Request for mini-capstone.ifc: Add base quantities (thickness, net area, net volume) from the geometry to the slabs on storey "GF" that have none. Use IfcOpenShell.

First a look at what the model holds.

```python
import ifcopenshell
import ifcopenshell.util.element
import ifcopenshell.util.unit

model = ifcopenshell.open("mini-capstone.ifc")
print(model.schema)
for unit_type in ("LENGTHUNIT", "AREAUNIT", "VOLUMEUNIT"):
    print(unit_type, ifcopenshell.util.unit.calculate_unit_scale(model, unit_type))
storey = next(s for s in model.by_type("IfcBuildingStorey") if s.Name == "GF")
slabs = [e for e in ifcopenshell.util.element.get_decomposition(storey) if e.is_a("IfcSlab")]
for e in sorted(slabs, key=lambda e: e.id()):
    print(e.id(), e.is_a(), e.Name, list(ifcopenshell.util.element.get_psets(e, qtos_only=True)), sep=" | ")
```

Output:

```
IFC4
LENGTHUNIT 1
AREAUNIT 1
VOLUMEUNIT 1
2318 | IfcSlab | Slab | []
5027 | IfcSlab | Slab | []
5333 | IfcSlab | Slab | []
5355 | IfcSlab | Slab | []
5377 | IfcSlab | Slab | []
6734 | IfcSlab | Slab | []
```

```python
import ifcopenshell
import ifcopenshell.api.pset
import ifcopenshell.geom
import ifcopenshell.util.element
import ifcopenshell.util.shape
import ifcopenshell.util.unit

model = ifcopenshell.open("mini-capstone.ifc")
unit_scale = ifcopenshell.util.unit.calculate_unit_scale(model)
area_scale = ifcopenshell.util.unit.calculate_unit_scale(model, "AREAUNIT")
volume_scale = ifcopenshell.util.unit.calculate_unit_scale(model, "VOLUMEUNIT")
settings = ifcopenshell.geom.settings()

storey = next(s for s in model.by_type("IfcBuildingStorey") if s.Name == "GF")
slabs = [e for e in ifcopenshell.util.element.get_decomposition(storey) if e.is_a("IfcSlab")]

for e in sorted(slabs, key=lambda e: e.id()):
    if ifcopenshell.util.element.get_psets(e, qtos_only=True, should_inherit=False):
        continue
    # Geometry comes back in metres, in the element's own axes.
    shape = ifcopenshell.geom.create_shape(settings, e)
    values = {
        "Width": ifcopenshell.util.shape.get_z(shape.geometry) / unit_scale,
        "NetArea": ifcopenshell.util.shape.get_footprint_area(shape.geometry) / area_scale,
        "NetVolume": ifcopenshell.util.shape.get_volume(shape.geometry) / volume_scale,
    }
    qto = ifcopenshell.api.pset.add_qto(model, product=e, name="Qto_SlabBaseQuantities")
    ifcopenshell.api.pset.edit_qto(model, qto=qto, properties=values)
    print(e.id(), {k: round(v, 3) for k, v in values.items()})

model.write("mini-capstone_edited.ifc")
```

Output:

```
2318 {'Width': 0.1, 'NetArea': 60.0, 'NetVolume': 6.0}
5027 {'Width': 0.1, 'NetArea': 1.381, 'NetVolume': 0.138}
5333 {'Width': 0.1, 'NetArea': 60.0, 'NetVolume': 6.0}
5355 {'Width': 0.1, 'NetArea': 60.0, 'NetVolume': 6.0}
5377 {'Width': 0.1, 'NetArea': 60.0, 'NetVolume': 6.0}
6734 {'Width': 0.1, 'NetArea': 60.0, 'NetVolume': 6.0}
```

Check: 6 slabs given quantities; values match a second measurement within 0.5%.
